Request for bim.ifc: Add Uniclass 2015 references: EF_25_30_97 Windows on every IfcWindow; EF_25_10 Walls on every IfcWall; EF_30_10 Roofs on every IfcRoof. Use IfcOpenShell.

First a look at what the model holds.

```python
import ifcopenshell

model = ifcopenshell.open("bim.ifc")
print(model.schema)
print("classifications:", [c.Name for c in model.by_type("IfcClassification")])
for ifc_class in ("IfcDoor", "IfcRoof", "IfcStair", "IfcWall", "IfcWindow"):
    print(ifc_class, len(model.by_type(ifc_class)))
```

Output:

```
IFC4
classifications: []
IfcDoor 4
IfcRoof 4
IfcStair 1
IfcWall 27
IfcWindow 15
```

```python
import ifcopenshell
import ifcopenshell.api.classification

model = ifcopenshell.open("bim.ifc")

system = ifcopenshell.api.classification.add_classification(model, classification="Uniclass 2015")

codes = {
    "IfcWindow": ("EF_25_30_97", "Windows"),
    "IfcWall": ("EF_25_10", "Walls"),
    "IfcRoof": ("EF_30_10", "Roofs"),
}
for ifc_class, (code, name) in codes.items():
    products = model.by_type(ifc_class)
    ifcopenshell.api.classification.add_reference(
        model, products=products, classification=system, identification=code, name=name
    )
    print(code, len(products))

model.write("bim_v2.ifc")
```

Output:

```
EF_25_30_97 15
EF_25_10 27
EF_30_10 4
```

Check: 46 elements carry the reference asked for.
